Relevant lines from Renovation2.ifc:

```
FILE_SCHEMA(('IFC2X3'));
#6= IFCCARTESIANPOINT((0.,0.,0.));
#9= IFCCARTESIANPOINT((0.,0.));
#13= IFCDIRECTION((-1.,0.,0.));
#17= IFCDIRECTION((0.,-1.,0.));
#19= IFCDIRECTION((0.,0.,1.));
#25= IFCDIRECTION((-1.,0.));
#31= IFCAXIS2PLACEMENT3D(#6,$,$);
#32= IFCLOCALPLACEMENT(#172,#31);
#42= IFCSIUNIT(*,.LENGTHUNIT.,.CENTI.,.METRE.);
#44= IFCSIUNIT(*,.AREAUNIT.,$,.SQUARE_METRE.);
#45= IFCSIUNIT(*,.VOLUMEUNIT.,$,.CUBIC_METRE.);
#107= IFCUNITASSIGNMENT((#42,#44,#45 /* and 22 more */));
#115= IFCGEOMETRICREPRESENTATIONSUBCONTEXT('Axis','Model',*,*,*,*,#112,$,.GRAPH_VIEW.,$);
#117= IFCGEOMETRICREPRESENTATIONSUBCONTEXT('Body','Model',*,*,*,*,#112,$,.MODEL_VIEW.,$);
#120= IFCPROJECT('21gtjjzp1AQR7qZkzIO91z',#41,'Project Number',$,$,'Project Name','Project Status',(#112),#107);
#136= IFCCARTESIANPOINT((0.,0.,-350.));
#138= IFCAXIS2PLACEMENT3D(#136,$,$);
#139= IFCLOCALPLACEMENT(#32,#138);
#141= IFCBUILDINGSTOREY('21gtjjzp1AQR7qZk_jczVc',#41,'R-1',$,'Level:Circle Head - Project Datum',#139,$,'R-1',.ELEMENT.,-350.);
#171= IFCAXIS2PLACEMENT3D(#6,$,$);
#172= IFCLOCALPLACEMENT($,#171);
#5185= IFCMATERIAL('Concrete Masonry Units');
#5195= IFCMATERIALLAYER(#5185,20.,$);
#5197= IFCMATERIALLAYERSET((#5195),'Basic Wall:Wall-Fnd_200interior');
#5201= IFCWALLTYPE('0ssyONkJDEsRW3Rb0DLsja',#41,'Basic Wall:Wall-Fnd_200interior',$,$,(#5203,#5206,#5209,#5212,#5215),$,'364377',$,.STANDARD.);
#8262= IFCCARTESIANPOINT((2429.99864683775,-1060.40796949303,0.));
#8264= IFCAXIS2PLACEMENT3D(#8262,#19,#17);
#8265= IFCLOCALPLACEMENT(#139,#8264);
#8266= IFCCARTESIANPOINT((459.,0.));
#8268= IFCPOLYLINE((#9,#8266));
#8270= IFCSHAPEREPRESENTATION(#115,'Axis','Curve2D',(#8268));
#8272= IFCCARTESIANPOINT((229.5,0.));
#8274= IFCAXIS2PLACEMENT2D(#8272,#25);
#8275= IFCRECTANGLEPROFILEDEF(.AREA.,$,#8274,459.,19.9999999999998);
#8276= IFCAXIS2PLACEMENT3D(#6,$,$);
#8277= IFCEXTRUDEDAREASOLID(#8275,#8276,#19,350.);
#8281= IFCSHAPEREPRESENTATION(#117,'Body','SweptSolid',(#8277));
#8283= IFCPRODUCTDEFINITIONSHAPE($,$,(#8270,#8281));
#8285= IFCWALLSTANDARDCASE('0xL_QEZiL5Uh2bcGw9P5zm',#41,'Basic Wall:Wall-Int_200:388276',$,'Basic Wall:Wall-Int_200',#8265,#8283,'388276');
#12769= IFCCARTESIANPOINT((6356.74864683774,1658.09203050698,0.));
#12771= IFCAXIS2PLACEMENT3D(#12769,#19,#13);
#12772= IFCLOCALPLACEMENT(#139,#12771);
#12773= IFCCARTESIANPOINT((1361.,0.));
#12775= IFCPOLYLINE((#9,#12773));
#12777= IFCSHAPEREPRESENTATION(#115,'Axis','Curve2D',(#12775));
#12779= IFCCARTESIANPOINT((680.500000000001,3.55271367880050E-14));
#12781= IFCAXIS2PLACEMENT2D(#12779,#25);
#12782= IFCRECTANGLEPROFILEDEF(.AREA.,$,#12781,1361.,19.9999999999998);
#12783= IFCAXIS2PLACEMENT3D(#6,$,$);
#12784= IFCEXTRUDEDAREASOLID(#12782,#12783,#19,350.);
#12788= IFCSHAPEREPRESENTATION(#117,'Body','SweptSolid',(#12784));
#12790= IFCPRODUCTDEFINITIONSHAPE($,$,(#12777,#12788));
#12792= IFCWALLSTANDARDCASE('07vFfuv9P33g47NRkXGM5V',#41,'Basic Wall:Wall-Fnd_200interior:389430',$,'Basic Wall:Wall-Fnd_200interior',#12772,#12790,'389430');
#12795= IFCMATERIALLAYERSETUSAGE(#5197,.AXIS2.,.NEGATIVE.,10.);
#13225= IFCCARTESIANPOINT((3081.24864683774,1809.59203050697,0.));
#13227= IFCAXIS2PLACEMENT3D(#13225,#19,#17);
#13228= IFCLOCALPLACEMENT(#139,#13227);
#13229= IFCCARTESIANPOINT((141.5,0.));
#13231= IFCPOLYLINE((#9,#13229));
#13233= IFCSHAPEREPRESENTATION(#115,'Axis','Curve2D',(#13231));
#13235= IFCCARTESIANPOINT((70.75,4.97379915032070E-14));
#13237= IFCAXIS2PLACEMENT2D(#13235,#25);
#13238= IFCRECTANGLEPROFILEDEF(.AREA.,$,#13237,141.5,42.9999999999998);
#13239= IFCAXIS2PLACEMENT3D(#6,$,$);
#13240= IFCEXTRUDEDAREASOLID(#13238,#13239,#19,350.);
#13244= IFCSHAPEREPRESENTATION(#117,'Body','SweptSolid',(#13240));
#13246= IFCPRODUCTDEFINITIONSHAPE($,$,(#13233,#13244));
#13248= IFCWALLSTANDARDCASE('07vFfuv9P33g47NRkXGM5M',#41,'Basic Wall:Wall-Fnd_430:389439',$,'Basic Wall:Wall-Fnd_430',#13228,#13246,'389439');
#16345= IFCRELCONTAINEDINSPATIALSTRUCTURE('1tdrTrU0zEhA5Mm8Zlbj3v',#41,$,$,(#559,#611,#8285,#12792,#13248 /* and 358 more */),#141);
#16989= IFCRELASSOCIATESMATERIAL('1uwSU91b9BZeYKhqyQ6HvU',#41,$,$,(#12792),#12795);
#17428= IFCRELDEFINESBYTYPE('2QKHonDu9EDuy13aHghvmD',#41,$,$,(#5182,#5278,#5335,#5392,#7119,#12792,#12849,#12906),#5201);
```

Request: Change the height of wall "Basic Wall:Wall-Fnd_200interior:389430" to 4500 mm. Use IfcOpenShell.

```python
import ifcopenshell
import ifcopenshell.geom
import ifcopenshell.util.representation
import ifcopenshell.util.shape
import ifcopenshell.util.unit

model = ifcopenshell.open("Renovation2.ifc")
unit_scale = ifcopenshell.util.unit.calculate_unit_scale(model)
settings = ifcopenshell.geom.settings()


def volume(element):
    """Net volume in cubic metres, openings subtracted."""
    shape = ifcopenshell.geom.create_shape(settings, element)
    return ifcopenshell.util.shape.get_volume(shape.geometry)


wall = model.by_guid("07vFfuv9P33g47NRkXGM5V")
before = volume(wall)

body = ifcopenshell.util.representation.get_representation(wall, "Model", "Body")
solid = body.Items[0]
old_height = solid.Depth
solid.Depth = 4.5 / unit_scale
after = volume(wall)

print(f"height {old_height:g} -> {solid.Depth:g}, volume {before:.3f} -> {after:.3f} m3")

model.write("Renovation2_v2.ifc")
```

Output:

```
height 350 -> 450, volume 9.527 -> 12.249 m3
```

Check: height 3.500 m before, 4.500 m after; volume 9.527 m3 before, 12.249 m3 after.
